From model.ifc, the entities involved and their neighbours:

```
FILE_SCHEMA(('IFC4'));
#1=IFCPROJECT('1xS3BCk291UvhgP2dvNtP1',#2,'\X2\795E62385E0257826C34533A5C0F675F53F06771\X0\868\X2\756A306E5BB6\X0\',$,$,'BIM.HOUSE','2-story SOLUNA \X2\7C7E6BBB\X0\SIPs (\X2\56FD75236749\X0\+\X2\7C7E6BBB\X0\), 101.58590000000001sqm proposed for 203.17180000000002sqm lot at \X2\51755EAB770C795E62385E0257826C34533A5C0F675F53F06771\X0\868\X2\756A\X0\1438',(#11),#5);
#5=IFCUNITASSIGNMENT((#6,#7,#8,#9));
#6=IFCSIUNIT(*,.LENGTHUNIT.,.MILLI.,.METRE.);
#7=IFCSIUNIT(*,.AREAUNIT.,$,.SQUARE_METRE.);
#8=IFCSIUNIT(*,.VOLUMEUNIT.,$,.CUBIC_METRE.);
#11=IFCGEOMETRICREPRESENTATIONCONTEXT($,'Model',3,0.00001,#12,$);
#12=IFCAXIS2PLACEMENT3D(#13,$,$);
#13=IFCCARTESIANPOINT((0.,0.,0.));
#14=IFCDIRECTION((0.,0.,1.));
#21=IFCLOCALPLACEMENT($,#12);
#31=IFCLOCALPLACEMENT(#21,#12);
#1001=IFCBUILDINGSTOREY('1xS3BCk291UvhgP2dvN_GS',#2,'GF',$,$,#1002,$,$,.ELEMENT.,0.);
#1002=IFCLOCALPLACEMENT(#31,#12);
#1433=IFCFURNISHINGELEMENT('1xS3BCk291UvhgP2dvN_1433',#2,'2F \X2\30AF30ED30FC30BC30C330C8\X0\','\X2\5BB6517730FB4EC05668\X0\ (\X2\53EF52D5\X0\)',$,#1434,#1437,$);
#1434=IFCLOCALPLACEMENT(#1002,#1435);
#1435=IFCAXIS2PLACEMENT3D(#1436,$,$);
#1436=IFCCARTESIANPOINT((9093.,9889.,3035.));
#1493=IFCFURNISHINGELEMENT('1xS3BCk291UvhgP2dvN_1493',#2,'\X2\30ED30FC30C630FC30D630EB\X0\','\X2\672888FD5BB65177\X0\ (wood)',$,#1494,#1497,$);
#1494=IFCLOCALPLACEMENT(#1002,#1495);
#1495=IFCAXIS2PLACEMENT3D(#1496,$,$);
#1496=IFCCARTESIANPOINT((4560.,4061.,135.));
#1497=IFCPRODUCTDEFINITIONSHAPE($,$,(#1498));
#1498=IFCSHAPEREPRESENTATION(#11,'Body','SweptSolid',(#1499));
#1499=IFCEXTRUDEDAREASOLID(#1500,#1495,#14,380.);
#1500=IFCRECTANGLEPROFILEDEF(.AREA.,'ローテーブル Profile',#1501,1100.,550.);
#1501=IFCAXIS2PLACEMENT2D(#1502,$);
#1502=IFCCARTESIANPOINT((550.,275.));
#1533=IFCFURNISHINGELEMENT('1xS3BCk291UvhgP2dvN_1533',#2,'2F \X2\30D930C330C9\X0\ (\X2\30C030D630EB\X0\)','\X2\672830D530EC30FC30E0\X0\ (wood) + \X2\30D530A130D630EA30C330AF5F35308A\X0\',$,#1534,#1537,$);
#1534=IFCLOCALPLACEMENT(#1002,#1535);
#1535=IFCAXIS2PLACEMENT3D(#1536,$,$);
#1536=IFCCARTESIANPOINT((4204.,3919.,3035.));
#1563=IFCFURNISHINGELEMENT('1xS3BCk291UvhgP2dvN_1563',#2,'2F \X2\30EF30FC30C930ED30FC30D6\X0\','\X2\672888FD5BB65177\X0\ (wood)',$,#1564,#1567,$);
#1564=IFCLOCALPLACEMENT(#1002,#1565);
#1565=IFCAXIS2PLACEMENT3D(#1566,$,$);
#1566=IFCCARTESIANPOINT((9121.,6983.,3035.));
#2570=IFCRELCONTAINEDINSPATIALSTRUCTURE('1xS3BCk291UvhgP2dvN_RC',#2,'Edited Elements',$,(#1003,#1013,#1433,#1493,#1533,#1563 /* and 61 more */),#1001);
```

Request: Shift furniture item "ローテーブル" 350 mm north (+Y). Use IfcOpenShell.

```python
import ifcopenshell
import ifcopenshell.api.geometry
import ifcopenshell.util.placement
import ifcopenshell.util.unit

model = ifcopenshell.open("model.ifc")
unit_scale = ifcopenshell.util.unit.calculate_unit_scale(model)

item = model.by_guid("1xS3BCk291UvhgP2dvN_1493")
matrix = ifcopenshell.util.placement.get_local_placement(item.ObjectPlacement)
matrix[1, 3] += 0.35 / unit_scale
ifcopenshell.api.geometry.edit_object_placement(model, product=item, matrix=matrix, is_si=False)

print(ifcopenshell.util.placement.get_local_placement(item.ObjectPlacement).round(3) + 0.0)

model.write("model-out.ifc")
```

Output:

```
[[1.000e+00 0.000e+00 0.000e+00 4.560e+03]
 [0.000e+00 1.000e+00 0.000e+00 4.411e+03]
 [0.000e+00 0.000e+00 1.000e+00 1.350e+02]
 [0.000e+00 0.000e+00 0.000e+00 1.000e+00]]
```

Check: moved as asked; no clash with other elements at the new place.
